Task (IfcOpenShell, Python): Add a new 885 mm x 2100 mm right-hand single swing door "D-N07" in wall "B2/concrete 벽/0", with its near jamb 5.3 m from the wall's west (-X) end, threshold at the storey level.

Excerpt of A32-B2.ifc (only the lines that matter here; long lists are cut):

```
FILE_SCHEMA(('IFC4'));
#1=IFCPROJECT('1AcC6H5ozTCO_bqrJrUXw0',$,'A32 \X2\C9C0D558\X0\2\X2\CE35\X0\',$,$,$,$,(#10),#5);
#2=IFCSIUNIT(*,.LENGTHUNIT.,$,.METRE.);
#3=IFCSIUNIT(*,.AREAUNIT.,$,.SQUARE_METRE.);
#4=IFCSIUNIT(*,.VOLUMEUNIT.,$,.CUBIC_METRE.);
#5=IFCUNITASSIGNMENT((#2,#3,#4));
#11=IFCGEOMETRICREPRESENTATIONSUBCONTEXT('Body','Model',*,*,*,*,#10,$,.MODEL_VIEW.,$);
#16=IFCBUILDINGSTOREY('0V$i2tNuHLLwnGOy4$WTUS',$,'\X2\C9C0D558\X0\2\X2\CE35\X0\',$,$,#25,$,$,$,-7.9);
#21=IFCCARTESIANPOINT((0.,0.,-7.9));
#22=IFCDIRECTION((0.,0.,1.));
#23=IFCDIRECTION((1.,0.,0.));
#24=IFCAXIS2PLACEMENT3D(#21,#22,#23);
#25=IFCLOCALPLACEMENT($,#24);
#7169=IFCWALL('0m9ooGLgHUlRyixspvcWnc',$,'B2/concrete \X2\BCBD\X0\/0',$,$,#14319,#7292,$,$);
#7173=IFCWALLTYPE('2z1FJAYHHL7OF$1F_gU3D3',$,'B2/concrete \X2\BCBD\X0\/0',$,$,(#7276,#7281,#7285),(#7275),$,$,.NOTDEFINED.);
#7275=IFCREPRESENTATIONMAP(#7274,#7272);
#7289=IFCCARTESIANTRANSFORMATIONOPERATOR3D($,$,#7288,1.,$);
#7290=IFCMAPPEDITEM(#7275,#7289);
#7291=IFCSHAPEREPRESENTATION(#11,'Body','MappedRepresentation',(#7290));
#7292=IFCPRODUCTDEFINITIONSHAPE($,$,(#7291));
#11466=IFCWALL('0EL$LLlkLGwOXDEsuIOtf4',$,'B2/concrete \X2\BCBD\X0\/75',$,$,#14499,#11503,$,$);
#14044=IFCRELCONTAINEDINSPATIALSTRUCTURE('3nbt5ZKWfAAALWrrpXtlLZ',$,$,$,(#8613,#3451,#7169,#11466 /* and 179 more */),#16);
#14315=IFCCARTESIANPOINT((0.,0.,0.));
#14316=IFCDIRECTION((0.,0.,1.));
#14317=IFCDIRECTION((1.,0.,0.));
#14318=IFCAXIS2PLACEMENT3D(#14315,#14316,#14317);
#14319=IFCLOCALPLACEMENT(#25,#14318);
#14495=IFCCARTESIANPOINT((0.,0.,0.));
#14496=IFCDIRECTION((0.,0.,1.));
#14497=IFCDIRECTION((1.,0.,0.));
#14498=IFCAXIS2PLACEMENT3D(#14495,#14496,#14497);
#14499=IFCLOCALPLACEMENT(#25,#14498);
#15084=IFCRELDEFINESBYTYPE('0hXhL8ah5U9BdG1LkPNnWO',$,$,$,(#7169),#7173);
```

```python
import numpy as np
import ifcopenshell
import ifcopenshell.api.feature
import ifcopenshell.api.geometry
import ifcopenshell.api.root
import ifcopenshell.api.spatial
import ifcopenshell.geom
import ifcopenshell.util.element
import ifcopenshell.util.placement
import ifcopenshell.util.representation
import ifcopenshell.util.shape
import ifcopenshell.util.unit

model = ifcopenshell.open("A32-B2.ifc")
unit_scale = ifcopenshell.util.unit.calculate_unit_scale(model)
settings = ifcopenshell.geom.settings()


def volume(element):
    """Net volume in cubic metres, openings subtracted."""
    shape = ifcopenshell.geom.create_shape(settings, element)
    return ifcopenshell.util.shape.get_volume(shape.geometry)


wall = model.by_id(7169)
storey = ifcopenshell.util.element.get_container(wall, ifc_class="IfcBuildingStorey")
context = ifcopenshell.util.representation.get_context(model, "Model", "Body", "MODEL_VIEW")
before = volume(wall)

width, height, from_end, sill = 0.885, 2.1, 5.3, 0.0  # metres

# The wall runs along its own X axis, and the end named is its -X end.
wall_shape = ifcopenshell.geom.create_shape(settings, wall)
x, y, z = ifcopenshell.util.shape.get_vertices(wall_shape.geometry).T
start = x.min() + from_end
face, thickness = float(y.min()), float(y.max() - y.min())
wall_matrix = ifcopenshell.util.placement.get_local_placement(wall.ObjectPlacement)
level = ifcopenshell.util.placement.get_local_placement(storey.ObjectPlacement)[2, 3]


def in_wall(x, y):
    """Placement at x, y metres in the wall's axes, at sill height."""
    matrix = wall_matrix.copy()
    matrix[:, 3] = wall_matrix @ np.array([x / unit_scale, y / unit_scale, 0.0, 1.0])
    matrix[2, 3] = level + sill / unit_scale
    return matrix


# Opening: a box that overshoots both wall faces by 50 mm.
opening = ifcopenshell.api.root.create_entity(model, ifc_class="IfcOpeningElement", predefined_type="OPENING")
box = ifcopenshell.api.geometry.add_wall_representation(
    model, context=context, length=width, height=height, thickness=thickness + 0.1
)
ifcopenshell.api.geometry.assign_representation(model, product=opening, representation=box)
ifcopenshell.api.geometry.edit_object_placement(model, product=opening, matrix=in_wall(start, face - 0.05), is_si=False)
ifcopenshell.api.feature.add_feature(model, feature=opening, element=wall)

door = ifcopenshell.api.root.create_entity(model, ifc_class="IfcDoor", name="D-N07", predefined_type="DOOR")
door.OverallWidth, door.OverallHeight = width / unit_scale, height / unit_scale
door.OperationType = "SINGLE_SWING_RIGHT"
body = ifcopenshell.api.geometry.add_door_representation(
    model,
    context=context,
    overall_width=door.OverallWidth,
    overall_height=door.OverallHeight,
    operation_type="SINGLE_SWING_RIGHT",
    lining_properties={"LiningDepth": thickness / unit_scale, "ThresholdDepth": thickness / unit_scale},
)
ifcopenshell.api.geometry.assign_representation(model, product=door, representation=body)
ifcopenshell.api.spatial.assign_container(model, products=[door], relating_structure=storey)
ifcopenshell.api.feature.add_filling(model, opening=opening, element=door)

# The lining spans the wall, so the door starts at the wall face.
ifcopenshell.api.geometry.edit_object_placement(model, product=door, matrix=in_wall(start, face), is_si=False)

after = volume(wall)

print(f"wall volume {before:.3f} -> {after:.3f} m3")

model.write("A32-B2-out.ifc")
```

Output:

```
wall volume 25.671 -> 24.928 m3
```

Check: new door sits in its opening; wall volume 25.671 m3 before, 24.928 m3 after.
